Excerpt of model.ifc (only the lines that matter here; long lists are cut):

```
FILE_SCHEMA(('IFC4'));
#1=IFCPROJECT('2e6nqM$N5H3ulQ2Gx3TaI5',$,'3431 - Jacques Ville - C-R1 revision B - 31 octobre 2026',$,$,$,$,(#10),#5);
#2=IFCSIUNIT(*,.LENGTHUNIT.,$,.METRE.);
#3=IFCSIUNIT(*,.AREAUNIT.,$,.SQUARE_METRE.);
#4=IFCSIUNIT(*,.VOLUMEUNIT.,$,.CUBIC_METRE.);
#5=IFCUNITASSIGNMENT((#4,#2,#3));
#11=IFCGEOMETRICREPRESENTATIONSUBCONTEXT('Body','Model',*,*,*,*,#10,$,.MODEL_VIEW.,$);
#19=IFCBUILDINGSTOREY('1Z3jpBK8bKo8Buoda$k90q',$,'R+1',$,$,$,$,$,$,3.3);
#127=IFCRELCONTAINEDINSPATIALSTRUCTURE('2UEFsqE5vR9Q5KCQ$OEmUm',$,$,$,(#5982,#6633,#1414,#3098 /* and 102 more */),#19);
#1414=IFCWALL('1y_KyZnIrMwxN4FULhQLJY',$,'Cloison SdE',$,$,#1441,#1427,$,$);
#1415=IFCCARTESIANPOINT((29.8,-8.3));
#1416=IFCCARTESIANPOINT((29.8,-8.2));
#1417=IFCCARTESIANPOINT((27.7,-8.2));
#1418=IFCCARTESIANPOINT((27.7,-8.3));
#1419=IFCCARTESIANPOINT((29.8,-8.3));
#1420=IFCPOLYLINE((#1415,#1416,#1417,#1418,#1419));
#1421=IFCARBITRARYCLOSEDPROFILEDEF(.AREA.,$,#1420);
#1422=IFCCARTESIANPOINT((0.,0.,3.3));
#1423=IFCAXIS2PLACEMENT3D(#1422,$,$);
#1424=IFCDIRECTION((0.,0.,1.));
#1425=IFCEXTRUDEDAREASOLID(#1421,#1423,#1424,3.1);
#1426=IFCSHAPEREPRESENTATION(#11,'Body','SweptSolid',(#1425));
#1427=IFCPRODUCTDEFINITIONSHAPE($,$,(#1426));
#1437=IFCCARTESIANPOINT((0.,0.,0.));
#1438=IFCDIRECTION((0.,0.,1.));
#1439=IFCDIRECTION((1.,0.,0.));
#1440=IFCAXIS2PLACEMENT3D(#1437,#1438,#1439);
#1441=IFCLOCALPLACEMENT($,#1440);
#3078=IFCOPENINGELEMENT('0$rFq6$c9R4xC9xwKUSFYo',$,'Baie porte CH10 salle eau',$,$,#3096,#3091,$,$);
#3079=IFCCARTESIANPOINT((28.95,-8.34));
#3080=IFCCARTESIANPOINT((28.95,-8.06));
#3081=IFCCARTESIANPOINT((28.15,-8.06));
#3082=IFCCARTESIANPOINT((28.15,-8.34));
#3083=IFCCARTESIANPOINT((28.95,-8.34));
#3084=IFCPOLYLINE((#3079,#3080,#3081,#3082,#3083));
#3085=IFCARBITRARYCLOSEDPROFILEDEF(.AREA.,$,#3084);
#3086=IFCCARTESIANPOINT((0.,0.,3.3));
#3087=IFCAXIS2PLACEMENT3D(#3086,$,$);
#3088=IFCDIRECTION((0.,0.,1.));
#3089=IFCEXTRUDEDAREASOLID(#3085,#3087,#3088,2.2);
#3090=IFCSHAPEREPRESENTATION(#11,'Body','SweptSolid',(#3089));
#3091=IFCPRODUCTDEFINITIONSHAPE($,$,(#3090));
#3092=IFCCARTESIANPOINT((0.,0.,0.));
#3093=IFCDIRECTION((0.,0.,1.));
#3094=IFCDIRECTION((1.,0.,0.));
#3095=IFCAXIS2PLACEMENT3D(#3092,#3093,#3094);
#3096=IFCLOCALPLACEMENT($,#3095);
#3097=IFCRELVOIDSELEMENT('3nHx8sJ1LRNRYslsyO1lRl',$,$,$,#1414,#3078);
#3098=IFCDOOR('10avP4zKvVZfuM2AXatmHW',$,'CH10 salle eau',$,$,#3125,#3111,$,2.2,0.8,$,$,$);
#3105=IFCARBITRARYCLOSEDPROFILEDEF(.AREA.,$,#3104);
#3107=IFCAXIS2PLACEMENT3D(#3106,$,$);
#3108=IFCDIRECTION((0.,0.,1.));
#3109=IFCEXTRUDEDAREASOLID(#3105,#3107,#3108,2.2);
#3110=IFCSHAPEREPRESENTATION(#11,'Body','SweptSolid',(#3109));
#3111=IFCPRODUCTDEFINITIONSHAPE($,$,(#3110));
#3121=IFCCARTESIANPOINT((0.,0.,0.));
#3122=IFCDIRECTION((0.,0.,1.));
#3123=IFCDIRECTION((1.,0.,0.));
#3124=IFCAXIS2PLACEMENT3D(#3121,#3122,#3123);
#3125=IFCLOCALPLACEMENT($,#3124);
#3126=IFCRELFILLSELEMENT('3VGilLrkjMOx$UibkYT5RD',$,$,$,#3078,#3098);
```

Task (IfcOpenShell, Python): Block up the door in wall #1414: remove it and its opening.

```python
import ifcopenshell
import ifcopenshell.api.feature
import ifcopenshell.api.root
import ifcopenshell.geom
import ifcopenshell.util.shape

model = ifcopenshell.open("model.ifc")
settings = ifcopenshell.geom.settings()


def volume(element):
    """Net volume in cubic metres, openings subtracted."""
    shape = ifcopenshell.geom.create_shape(settings, element)
    return ifcopenshell.util.shape.get_volume(shape.geometry)


door = model.by_id(3098)
opening = door.FillsVoids[0].RelatingOpeningElement
wall = opening.VoidsElements[0].RelatingBuildingElement
before = volume(wall)

ifcopenshell.api.root.remove_product(model, product=door)
ifcopenshell.api.feature.remove_feature(model, feature=opening)

after = volume(wall)

print(f"wall volume {before:.3f} -> {after:.3f} m3")

model.write("model_updated.ifc")
```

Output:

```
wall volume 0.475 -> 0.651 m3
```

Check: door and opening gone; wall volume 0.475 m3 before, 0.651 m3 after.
